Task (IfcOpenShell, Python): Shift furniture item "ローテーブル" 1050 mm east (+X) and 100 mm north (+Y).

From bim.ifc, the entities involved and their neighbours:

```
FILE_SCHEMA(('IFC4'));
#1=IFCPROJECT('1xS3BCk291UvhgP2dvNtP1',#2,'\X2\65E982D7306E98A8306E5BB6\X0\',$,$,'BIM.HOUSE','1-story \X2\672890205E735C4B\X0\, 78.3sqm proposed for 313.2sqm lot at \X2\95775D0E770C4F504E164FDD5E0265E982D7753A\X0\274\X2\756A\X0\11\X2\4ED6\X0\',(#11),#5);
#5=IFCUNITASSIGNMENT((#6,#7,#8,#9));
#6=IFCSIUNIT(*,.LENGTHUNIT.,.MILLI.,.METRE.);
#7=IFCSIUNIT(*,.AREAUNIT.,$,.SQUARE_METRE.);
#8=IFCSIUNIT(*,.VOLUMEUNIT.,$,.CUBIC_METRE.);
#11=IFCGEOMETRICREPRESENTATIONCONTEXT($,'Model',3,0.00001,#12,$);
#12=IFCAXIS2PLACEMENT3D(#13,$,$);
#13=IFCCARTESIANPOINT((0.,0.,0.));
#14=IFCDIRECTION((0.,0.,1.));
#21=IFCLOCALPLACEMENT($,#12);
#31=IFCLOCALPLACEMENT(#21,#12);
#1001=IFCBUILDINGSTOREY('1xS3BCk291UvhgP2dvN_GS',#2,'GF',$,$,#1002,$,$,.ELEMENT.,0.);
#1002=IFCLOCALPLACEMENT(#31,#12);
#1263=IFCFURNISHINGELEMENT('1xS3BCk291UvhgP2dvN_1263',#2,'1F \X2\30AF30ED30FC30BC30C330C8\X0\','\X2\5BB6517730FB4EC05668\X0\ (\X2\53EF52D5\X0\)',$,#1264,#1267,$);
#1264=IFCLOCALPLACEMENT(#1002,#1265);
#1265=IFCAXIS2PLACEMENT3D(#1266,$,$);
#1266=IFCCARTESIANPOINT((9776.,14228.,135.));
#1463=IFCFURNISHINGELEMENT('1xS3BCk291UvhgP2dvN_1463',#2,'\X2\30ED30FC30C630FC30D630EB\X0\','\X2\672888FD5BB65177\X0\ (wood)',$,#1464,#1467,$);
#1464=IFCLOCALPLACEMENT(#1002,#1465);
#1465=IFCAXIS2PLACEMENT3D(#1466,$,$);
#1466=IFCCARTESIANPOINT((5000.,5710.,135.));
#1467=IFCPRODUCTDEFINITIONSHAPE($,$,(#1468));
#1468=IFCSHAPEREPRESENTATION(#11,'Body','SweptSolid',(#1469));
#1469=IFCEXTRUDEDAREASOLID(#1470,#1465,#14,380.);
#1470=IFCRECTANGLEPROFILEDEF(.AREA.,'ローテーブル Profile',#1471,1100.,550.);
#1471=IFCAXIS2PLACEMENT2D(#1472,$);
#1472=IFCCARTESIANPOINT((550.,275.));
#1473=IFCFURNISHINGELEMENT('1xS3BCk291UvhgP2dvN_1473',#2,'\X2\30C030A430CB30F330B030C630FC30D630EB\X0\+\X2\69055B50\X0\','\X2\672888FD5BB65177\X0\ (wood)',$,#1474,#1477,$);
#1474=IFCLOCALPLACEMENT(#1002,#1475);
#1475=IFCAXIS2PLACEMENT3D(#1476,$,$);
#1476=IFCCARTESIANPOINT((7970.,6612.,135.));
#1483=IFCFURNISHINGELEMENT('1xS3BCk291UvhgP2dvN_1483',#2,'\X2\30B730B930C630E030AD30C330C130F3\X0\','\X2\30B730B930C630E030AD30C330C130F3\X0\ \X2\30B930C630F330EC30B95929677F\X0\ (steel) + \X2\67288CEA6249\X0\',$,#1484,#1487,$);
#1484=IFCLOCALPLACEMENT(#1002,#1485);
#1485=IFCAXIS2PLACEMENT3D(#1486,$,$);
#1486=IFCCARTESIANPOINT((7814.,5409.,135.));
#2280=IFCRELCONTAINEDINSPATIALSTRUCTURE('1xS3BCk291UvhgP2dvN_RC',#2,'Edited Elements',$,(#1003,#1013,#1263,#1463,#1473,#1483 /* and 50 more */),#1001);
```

```python
import ifcopenshell
import ifcopenshell.api.geometry
import ifcopenshell.util.placement
import ifcopenshell.util.unit

model = ifcopenshell.open("bim.ifc")
unit_scale = ifcopenshell.util.unit.calculate_unit_scale(model)

item = model.by_guid("1xS3BCk291UvhgP2dvN_1463")
matrix = ifcopenshell.util.placement.get_local_placement(item.ObjectPlacement)
matrix[0, 3] += 1.05 / unit_scale
matrix[1, 3] += 0.1 / unit_scale
ifcopenshell.api.geometry.edit_object_placement(model, product=item, matrix=matrix, is_si=False)

print(ifcopenshell.util.placement.get_local_placement(item.ObjectPlacement).round(3) + 0.0)

model.write("bim-out.ifc")
```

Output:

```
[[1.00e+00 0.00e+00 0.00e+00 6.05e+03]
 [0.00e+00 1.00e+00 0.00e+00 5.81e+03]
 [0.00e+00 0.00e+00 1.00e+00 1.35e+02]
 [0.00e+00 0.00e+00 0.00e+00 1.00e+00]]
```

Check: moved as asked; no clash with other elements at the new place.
